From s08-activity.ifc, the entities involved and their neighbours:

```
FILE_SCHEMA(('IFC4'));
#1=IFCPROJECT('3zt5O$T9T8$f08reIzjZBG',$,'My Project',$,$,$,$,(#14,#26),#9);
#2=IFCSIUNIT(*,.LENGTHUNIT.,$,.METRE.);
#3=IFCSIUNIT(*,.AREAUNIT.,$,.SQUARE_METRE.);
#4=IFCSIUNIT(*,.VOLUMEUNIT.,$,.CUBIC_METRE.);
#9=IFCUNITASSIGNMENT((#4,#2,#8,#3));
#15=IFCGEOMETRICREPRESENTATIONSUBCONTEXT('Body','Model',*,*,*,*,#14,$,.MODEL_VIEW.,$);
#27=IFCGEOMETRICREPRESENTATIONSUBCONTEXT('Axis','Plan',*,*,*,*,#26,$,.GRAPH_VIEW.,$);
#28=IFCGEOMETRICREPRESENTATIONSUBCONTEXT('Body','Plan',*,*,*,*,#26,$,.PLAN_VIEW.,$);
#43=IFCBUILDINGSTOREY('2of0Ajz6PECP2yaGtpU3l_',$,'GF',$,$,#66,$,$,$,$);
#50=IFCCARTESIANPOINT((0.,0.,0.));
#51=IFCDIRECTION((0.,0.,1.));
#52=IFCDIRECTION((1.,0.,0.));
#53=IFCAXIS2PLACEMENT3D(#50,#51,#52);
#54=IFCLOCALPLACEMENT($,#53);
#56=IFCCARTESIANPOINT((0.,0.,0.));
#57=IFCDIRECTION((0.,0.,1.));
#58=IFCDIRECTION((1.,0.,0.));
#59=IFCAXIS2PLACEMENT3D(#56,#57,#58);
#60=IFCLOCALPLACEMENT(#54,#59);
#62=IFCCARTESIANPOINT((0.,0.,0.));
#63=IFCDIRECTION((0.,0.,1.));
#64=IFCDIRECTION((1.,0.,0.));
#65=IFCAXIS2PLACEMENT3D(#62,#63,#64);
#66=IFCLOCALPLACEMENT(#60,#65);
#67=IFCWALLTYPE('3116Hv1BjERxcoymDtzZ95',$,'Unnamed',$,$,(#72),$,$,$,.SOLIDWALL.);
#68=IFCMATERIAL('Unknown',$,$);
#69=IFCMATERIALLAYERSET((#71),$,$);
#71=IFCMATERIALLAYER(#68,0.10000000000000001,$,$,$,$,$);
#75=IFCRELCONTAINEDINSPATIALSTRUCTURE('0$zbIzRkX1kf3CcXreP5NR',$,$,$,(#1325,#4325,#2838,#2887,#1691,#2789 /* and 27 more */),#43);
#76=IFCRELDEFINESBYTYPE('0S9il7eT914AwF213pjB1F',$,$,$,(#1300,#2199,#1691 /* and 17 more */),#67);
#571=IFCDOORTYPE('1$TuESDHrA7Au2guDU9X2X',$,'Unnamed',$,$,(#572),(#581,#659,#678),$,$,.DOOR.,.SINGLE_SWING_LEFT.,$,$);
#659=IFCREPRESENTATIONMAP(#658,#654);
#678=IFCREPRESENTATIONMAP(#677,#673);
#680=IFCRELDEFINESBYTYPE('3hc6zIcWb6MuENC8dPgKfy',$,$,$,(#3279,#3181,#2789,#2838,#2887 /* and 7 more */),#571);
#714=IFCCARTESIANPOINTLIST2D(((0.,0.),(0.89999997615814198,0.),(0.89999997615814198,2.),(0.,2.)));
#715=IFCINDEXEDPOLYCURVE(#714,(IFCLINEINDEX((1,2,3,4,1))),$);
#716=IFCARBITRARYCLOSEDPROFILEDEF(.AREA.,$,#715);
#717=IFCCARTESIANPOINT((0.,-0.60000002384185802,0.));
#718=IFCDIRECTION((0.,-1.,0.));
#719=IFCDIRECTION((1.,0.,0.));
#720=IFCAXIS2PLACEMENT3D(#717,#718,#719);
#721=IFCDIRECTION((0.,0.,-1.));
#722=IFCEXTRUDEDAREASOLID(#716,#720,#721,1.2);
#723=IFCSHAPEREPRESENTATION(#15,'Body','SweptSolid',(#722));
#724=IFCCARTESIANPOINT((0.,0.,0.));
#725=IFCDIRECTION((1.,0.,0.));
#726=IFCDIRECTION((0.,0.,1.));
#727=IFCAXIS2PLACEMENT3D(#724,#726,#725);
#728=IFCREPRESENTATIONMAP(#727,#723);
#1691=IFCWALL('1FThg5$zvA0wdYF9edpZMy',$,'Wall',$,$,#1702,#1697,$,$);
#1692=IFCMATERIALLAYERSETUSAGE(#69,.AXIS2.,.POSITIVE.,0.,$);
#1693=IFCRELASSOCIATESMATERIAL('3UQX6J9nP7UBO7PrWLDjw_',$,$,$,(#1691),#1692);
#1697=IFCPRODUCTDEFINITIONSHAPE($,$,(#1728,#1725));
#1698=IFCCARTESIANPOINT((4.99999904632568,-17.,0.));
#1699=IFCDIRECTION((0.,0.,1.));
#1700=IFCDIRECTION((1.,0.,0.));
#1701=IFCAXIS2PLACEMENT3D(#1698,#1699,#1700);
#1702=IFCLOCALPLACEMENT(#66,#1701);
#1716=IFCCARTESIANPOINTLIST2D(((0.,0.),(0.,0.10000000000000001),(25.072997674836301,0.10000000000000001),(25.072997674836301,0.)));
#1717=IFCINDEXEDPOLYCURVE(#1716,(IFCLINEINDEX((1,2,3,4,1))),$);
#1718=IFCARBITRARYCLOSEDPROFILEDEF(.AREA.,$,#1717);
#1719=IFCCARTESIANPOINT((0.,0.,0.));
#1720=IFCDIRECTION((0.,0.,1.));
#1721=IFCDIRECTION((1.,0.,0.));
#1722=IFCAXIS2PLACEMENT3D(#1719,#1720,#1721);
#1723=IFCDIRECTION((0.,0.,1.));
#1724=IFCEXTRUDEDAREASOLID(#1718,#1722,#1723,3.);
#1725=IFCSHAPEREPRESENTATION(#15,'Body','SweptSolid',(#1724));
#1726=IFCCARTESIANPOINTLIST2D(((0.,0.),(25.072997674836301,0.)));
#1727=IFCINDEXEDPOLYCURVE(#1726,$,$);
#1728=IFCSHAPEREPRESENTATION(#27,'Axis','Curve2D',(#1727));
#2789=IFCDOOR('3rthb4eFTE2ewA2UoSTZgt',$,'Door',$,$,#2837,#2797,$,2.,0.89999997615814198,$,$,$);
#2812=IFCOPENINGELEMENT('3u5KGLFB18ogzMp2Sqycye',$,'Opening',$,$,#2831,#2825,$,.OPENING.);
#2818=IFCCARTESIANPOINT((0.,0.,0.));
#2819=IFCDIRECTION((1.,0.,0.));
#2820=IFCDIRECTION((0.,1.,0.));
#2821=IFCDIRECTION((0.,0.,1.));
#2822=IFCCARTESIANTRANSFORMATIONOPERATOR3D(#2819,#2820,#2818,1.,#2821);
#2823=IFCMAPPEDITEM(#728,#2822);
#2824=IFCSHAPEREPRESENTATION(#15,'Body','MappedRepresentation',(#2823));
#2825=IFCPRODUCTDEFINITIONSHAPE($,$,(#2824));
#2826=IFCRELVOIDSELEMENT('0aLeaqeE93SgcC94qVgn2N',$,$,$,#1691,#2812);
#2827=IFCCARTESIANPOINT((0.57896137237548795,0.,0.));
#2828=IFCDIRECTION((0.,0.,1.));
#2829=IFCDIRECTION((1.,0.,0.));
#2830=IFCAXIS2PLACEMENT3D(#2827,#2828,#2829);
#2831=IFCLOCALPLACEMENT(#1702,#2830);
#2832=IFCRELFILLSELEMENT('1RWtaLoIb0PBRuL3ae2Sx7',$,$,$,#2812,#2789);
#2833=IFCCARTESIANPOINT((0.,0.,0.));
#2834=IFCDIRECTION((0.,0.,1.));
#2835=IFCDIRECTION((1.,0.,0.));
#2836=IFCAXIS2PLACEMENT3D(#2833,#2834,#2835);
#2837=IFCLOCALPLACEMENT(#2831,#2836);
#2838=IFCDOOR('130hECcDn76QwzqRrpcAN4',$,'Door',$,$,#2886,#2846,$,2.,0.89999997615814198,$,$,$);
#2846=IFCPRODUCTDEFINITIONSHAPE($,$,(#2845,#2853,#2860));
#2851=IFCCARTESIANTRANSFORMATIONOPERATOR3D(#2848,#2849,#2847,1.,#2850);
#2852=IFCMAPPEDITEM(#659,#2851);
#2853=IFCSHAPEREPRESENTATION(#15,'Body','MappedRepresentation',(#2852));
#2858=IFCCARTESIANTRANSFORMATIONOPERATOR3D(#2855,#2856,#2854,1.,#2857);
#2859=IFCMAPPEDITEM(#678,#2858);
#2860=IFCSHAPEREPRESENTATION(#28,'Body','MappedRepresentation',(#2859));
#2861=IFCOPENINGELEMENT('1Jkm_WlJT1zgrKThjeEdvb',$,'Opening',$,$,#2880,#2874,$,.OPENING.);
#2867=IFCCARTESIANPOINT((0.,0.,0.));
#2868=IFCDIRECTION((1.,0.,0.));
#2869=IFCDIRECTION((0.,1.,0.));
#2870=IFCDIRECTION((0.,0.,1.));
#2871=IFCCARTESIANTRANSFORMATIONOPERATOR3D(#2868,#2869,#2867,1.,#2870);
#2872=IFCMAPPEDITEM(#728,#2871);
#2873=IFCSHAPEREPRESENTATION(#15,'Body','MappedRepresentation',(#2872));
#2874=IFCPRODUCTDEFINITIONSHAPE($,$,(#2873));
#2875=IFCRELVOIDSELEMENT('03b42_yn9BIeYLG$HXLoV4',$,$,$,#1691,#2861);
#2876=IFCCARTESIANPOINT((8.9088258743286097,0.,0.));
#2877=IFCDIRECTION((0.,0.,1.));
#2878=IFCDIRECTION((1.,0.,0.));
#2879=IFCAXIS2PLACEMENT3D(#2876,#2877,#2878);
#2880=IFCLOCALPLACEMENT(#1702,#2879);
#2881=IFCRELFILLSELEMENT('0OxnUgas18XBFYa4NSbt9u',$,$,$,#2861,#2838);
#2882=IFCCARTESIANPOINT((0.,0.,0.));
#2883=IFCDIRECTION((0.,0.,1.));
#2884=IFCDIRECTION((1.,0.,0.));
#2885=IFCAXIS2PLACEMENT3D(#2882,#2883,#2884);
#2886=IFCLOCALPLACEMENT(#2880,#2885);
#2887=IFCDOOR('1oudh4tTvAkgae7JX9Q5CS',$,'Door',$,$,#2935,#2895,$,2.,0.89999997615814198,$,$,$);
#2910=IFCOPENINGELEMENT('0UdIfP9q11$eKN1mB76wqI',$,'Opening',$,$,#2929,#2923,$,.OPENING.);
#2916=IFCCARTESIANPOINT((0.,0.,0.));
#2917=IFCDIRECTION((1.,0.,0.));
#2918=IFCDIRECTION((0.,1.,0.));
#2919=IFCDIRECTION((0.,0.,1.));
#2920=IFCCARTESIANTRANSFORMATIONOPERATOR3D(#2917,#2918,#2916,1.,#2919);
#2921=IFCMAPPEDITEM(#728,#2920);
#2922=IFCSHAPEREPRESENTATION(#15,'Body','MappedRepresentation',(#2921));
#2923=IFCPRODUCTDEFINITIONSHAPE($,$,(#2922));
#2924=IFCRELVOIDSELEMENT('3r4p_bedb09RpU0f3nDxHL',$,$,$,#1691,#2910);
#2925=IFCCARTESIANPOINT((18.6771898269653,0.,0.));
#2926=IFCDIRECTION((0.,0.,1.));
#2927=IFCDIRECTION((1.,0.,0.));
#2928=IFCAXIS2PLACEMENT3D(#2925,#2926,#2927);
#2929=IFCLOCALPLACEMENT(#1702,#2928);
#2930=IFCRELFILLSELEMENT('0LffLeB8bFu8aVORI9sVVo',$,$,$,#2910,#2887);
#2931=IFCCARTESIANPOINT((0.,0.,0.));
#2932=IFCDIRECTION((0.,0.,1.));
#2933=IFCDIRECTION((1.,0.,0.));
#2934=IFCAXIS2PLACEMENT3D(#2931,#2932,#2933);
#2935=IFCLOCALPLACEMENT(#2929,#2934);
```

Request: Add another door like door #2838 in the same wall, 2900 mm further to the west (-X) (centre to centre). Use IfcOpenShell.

```python
import ifcopenshell
import ifcopenshell.api.feature
import ifcopenshell.api.geometry
import ifcopenshell.api.root
import ifcopenshell.geom
import ifcopenshell.util.element
import ifcopenshell.util.placement
import ifcopenshell.util.shape
import ifcopenshell.util.unit

model = ifcopenshell.open("s08-activity.ifc")
unit_scale = ifcopenshell.util.unit.calculate_unit_scale(model)
settings = ifcopenshell.geom.settings()


def volume(element):
    """Net volume in cubic metres, openings subtracted."""
    shape = ifcopenshell.geom.create_shape(settings, element)
    return ifcopenshell.util.shape.get_volume(shape.geometry)


door = model.by_id(2838)
opening = door.FillsVoids[0].RelatingOpeningElement
wall = opening.VoidsElements[0].RelatingBuildingElement
before = volume(wall)
shift = ifcopenshell.util.placement.get_local_placement(wall.ObjectPlacement)[:3, 0] * -2.9 / unit_scale

# copy_class copies the void relationship, type, container and properties, but no geometry.
new_opening = ifcopenshell.api.root.copy_class(model, product=opening)
new_opening.Representation = ifcopenshell.util.element.copy_deep(
    model, opening.Representation, exclude=["IfcGeometricRepresentationContext", "IfcRepresentationMap"]
)
new_door = ifcopenshell.api.root.copy_class(model, product=door)
new_door.Representation = ifcopenshell.util.element.copy_deep(
    model, door.Representation, exclude=["IfcGeometricRepresentationContext", "IfcRepresentationMap"]
)
ifcopenshell.api.feature.add_filling(model, opening=new_opening, element=new_door)

for old, new in ((opening, new_opening), (door, new_door)):
    matrix = ifcopenshell.util.placement.get_local_placement(old.ObjectPlacement)
    matrix[:3, 3] += shift
    ifcopenshell.api.geometry.edit_object_placement(model, product=new, matrix=matrix, is_si=False)

after = volume(wall)

print(f"wall volume {before:.3f} -> {after:.3f} m3")

model.write("s08-activity_edited.ifc")
```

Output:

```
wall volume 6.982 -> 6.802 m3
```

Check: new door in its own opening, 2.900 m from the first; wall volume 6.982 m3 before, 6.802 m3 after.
